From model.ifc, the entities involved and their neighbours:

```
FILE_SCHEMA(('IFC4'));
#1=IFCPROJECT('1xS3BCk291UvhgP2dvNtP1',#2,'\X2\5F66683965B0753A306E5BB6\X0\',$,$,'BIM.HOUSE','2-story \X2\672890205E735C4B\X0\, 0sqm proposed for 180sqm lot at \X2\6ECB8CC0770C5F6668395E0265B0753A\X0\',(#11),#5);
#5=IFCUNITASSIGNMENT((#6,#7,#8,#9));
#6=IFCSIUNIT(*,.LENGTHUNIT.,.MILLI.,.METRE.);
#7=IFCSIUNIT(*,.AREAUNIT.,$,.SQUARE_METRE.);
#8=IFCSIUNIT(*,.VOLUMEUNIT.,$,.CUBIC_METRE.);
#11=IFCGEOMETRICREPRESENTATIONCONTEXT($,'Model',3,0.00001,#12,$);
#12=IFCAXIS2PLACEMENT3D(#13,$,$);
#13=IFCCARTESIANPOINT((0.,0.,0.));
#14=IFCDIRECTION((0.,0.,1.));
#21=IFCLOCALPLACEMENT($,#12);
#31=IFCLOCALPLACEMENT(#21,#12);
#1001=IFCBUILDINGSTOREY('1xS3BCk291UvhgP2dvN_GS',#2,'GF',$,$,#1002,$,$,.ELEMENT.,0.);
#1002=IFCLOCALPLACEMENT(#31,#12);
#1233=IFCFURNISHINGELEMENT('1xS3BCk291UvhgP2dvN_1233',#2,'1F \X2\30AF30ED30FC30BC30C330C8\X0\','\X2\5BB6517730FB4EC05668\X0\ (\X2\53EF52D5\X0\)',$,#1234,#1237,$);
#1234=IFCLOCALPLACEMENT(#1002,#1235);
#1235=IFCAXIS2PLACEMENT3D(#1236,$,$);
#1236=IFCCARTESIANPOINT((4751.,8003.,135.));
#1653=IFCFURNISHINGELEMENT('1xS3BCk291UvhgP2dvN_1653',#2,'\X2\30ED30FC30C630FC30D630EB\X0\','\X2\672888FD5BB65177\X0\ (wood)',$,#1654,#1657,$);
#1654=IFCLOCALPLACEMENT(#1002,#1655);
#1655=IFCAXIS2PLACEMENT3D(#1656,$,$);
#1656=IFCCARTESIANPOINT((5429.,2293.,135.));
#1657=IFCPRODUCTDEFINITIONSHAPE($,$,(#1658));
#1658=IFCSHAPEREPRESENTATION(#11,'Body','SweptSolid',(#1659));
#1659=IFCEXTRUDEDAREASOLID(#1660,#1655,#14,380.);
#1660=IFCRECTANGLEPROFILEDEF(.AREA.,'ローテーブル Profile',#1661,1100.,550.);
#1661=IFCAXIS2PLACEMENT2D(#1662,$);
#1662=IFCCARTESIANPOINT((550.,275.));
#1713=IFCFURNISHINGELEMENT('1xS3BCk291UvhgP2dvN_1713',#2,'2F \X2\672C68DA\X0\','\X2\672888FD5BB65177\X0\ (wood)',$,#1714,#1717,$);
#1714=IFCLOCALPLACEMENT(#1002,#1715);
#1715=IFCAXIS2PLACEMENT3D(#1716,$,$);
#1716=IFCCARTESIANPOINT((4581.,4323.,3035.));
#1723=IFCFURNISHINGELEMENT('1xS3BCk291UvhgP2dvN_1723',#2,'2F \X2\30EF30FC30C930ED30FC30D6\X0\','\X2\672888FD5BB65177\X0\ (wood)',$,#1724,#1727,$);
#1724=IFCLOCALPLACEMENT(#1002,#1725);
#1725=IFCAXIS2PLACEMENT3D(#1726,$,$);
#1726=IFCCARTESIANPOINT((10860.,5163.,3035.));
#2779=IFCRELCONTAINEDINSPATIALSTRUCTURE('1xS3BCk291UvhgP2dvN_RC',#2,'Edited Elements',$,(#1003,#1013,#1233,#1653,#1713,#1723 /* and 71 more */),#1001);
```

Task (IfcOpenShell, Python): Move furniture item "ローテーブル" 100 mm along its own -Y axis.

```python
import ifcopenshell
import ifcopenshell.api.geometry
import ifcopenshell.util.placement
import ifcopenshell.util.unit

model = ifcopenshell.open("model.ifc")
unit_scale = ifcopenshell.util.unit.calculate_unit_scale(model)

item = model.by_guid("1xS3BCk291UvhgP2dvN_1653")
matrix = ifcopenshell.util.placement.get_local_placement(item.ObjectPlacement)
matrix[:3, 3] -= matrix[:3, 1] * 0.1 / unit_scale
ifcopenshell.api.geometry.edit_object_placement(model, product=item, matrix=matrix, is_si=False)

print(ifcopenshell.util.placement.get_local_placement(item.ObjectPlacement).round(3) + 0.0)

model.write("model_rev.ifc")
```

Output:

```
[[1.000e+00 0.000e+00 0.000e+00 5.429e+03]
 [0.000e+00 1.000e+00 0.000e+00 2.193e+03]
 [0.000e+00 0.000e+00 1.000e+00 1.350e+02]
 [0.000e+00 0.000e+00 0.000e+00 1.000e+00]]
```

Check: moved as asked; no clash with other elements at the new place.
